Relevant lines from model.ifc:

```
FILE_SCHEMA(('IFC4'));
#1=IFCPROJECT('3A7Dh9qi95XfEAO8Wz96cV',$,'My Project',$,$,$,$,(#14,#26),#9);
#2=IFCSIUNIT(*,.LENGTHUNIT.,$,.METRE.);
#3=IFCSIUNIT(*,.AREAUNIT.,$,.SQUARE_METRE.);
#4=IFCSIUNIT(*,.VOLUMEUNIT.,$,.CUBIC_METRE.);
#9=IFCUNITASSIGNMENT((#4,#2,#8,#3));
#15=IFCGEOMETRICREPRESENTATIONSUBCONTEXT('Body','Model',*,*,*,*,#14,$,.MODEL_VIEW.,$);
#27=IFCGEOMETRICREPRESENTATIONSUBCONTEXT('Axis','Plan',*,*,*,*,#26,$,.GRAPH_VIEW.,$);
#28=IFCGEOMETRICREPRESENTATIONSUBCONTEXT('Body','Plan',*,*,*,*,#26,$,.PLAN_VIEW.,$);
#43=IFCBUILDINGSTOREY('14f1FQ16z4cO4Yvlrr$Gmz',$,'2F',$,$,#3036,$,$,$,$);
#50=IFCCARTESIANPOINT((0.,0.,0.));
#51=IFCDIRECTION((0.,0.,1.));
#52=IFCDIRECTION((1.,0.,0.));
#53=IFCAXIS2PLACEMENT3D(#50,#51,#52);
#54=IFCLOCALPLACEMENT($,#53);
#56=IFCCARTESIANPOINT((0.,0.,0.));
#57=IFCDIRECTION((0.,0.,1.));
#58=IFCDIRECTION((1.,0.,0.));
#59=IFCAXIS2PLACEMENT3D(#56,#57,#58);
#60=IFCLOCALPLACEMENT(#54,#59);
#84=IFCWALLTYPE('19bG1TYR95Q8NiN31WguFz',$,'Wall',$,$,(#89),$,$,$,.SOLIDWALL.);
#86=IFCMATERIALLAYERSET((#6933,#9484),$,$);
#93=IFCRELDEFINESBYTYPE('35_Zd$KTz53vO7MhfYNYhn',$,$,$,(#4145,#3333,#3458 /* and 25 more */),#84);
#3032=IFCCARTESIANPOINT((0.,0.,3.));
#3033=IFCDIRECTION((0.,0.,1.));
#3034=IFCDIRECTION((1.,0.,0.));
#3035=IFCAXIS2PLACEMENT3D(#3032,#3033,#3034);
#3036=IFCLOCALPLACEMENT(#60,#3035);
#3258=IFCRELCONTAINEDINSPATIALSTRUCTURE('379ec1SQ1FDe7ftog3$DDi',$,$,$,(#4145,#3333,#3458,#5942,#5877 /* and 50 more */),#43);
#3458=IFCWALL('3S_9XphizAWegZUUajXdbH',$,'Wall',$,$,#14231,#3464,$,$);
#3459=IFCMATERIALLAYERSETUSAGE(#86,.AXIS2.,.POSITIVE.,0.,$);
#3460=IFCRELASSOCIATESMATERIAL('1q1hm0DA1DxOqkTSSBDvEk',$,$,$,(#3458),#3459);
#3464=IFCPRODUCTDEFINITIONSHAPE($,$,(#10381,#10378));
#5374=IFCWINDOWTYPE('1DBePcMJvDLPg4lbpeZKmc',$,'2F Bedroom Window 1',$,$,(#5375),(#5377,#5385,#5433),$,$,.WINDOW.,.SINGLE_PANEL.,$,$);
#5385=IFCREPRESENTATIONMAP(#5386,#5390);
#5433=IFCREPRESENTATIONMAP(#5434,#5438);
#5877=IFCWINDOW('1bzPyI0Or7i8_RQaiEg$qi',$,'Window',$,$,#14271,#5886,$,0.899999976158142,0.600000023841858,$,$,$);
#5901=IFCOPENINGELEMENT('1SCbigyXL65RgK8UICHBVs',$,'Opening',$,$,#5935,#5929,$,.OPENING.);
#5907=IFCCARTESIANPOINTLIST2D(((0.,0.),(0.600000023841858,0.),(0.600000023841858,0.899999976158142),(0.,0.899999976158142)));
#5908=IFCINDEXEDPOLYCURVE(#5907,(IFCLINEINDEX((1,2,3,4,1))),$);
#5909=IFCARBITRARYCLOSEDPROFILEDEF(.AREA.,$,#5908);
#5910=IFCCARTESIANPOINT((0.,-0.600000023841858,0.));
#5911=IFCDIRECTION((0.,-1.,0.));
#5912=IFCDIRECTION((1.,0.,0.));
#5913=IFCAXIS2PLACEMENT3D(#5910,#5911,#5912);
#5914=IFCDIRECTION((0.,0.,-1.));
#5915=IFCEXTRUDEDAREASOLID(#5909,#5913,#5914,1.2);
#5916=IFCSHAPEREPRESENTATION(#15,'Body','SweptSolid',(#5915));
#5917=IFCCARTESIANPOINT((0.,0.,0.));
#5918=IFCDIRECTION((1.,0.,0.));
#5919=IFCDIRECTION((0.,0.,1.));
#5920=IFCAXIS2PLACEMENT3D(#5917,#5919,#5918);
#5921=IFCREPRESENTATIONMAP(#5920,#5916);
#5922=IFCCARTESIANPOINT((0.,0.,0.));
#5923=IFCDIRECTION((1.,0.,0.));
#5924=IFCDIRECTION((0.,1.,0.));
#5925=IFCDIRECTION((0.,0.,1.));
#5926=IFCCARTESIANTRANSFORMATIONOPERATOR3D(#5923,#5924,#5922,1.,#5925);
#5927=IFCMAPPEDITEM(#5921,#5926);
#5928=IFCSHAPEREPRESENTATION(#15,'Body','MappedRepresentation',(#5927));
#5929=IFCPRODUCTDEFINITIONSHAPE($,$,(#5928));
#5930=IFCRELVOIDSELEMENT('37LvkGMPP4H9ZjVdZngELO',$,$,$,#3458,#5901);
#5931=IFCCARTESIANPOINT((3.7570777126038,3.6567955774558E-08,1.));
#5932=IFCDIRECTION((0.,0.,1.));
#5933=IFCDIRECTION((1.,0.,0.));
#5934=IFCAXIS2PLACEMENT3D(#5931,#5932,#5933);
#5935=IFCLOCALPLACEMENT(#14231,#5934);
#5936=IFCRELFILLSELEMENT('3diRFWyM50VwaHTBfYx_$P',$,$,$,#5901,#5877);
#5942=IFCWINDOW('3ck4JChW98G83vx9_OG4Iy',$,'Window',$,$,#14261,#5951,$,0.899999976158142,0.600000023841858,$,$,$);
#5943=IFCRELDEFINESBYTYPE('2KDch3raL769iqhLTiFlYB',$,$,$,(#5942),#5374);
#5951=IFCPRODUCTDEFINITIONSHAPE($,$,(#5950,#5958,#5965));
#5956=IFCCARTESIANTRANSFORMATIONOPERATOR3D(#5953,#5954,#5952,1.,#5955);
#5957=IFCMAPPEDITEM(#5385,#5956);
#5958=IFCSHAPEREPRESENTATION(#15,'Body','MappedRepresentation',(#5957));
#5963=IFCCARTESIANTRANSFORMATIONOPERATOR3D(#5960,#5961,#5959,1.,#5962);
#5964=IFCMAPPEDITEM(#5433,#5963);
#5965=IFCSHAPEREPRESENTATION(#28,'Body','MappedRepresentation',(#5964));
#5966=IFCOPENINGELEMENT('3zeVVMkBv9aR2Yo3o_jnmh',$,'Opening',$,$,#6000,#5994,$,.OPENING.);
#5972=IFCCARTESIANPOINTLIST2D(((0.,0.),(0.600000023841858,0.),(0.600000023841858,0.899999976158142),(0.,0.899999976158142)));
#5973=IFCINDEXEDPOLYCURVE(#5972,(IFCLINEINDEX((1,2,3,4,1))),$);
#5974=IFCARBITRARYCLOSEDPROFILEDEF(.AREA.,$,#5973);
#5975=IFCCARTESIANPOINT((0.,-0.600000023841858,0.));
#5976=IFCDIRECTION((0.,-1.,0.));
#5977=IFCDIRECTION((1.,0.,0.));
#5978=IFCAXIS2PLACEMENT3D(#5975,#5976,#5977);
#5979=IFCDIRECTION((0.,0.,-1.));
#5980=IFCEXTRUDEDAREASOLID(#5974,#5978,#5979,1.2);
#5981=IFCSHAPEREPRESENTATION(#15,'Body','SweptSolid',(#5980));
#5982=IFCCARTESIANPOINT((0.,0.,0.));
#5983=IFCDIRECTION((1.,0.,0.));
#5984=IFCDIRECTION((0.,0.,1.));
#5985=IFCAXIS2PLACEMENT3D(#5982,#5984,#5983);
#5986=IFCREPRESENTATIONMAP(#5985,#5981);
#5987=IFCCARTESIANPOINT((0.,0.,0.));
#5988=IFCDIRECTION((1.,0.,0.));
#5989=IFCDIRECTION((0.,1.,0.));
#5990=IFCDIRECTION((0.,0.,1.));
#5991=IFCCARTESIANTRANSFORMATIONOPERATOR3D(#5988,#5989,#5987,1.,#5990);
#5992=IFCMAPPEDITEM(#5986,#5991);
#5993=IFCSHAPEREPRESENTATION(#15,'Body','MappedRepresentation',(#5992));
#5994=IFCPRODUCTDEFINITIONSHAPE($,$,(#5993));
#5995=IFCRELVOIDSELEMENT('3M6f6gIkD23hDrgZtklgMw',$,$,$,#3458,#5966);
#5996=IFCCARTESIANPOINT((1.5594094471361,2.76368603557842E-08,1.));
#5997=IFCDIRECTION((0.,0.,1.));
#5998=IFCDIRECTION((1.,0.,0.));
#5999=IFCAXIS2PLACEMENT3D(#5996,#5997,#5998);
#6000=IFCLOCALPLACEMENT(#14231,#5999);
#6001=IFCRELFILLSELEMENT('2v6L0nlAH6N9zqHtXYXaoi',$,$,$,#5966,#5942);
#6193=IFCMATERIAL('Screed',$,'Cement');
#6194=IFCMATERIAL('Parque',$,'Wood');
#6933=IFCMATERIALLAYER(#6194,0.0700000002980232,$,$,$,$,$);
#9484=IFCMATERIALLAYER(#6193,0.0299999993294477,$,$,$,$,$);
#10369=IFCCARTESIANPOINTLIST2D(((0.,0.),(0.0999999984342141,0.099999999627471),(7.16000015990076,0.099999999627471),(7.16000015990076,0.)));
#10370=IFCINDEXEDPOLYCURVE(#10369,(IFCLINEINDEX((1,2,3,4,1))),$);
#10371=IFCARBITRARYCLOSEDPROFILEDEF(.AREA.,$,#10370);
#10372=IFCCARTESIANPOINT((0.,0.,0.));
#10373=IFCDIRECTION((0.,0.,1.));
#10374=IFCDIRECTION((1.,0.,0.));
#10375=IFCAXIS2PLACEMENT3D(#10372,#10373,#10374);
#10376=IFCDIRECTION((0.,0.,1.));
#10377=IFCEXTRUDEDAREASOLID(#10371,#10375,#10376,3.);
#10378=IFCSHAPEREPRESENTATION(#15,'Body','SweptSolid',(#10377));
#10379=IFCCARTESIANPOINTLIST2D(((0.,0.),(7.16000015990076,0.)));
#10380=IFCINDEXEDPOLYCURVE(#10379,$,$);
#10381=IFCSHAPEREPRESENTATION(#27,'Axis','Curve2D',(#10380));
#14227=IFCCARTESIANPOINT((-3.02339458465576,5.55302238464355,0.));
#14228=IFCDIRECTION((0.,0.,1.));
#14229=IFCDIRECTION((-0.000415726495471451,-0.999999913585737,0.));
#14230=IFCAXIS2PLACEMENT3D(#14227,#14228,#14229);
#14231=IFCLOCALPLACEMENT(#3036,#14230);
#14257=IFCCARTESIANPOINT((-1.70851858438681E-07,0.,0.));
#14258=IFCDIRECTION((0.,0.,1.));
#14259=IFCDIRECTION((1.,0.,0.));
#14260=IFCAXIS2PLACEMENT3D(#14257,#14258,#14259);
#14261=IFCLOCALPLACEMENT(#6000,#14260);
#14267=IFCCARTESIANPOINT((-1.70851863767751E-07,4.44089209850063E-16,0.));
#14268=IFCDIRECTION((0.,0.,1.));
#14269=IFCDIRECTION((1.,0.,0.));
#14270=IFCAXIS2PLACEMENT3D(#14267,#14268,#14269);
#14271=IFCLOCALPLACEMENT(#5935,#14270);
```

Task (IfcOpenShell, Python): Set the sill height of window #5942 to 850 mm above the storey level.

```python
import numpy as np
import ifcopenshell
import ifcopenshell.api.geometry
import ifcopenshell.geom
import ifcopenshell.util.element
import ifcopenshell.util.placement
import ifcopenshell.util.shape
import ifcopenshell.util.unit

model = ifcopenshell.open("model.ifc")
unit_scale = ifcopenshell.util.unit.calculate_unit_scale(model)

window = model.by_guid("3ck4JChW98G83vx9_OG4Iy")
opening = window.FillsVoids[0].RelatingOpeningElement
storey = ifcopenshell.util.element.get_container(window, ifc_class="IfcBuildingStorey")
level = ifcopenshell.util.placement.get_local_placement(storey.ObjectPlacement)[2, 3]

# The opening's origin need not be at the sill, so measure its lowest point.
shape = ifcopenshell.geom.create_shape(ifcopenshell.geom.settings(), opening)
bottom = ifcopenshell.util.shape.get_shape_bottom_elevation(shape, shape.geometry) / unit_scale
dz = level + 0.85 / unit_scale - bottom

shift = np.array([0.0, 0.0, dz])
# The window is placed relative to its opening, so it follows when the opening moves.
matrix = ifcopenshell.util.placement.get_local_placement(opening.ObjectPlacement)
matrix[:3, 3] += shift
ifcopenshell.api.geometry.edit_object_placement(
    model, product=opening, matrix=matrix, is_si=False, should_transform_children=True
)

print(f"moved by {dz * unit_scale:+.3f} m")

model.write("model-out.ifc")
```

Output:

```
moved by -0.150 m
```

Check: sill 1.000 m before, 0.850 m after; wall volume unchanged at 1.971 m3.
